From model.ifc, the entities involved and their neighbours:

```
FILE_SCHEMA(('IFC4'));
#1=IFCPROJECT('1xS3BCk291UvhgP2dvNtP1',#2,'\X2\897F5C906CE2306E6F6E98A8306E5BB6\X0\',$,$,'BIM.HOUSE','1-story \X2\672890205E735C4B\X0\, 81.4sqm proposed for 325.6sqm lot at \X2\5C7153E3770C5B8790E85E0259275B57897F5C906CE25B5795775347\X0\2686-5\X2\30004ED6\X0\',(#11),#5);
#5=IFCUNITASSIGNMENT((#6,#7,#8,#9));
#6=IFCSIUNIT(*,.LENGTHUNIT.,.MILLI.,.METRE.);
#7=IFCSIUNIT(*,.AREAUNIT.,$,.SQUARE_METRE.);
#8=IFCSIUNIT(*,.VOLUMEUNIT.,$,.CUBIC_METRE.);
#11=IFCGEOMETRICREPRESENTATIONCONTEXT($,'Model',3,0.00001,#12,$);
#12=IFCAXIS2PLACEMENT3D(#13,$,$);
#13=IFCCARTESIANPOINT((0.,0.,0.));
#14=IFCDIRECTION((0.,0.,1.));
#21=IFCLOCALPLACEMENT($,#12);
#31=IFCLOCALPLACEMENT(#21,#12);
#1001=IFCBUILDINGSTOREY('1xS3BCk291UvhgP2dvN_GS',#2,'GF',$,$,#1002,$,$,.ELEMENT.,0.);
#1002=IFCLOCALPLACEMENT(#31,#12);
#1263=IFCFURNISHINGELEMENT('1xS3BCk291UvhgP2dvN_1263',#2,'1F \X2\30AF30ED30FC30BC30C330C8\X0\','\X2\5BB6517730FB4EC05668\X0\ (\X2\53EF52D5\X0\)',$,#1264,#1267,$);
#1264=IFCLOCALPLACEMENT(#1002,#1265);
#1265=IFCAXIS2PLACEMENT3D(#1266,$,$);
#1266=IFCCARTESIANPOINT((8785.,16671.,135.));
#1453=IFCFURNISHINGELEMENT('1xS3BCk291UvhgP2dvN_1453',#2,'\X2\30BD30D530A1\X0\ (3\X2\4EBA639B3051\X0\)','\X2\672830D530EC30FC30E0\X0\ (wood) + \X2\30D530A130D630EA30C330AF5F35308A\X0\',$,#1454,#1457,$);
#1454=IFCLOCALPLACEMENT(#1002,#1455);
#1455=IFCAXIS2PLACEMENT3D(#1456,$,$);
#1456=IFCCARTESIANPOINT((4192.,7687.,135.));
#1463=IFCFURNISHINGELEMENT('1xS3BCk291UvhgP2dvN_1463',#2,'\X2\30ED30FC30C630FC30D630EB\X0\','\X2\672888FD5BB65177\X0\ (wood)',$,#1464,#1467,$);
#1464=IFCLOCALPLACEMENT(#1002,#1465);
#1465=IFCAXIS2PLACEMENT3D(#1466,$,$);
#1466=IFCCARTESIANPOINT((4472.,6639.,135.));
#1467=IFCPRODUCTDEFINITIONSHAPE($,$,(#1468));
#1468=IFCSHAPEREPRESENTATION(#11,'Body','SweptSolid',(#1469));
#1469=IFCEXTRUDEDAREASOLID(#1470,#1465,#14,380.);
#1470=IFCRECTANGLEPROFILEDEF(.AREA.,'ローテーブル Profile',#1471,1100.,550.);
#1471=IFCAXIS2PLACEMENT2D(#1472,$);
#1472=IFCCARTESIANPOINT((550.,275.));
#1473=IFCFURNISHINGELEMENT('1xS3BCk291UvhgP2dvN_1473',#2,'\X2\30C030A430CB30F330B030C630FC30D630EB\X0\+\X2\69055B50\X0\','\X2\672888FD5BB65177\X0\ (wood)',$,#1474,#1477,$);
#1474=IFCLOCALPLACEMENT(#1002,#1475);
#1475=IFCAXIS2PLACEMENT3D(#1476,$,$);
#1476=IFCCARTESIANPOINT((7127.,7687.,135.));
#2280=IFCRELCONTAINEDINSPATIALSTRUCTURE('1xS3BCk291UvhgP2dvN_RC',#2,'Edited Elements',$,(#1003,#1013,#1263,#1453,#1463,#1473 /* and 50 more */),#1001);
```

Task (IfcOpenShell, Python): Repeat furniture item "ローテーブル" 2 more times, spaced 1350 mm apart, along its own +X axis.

```python
import ifcopenshell
import ifcopenshell.api.geometry
import ifcopenshell.api.root
import ifcopenshell.util.element
import ifcopenshell.util.placement
import ifcopenshell.util.unit

model = ifcopenshell.open("model.ifc")
unit_scale = ifcopenshell.util.unit.calculate_unit_scale(model)


def reuse_history(source, copy):
    """copy_class also copies each property set's owner history, people and application; keep the originals."""
    for rel in copy.IsDefinedBy:
        if rel.is_a("IfcRelDefinesByProperties") and (history := rel.RelatingPropertyDefinition.OwnerHistory):
            rel.RelatingPropertyDefinition.OwnerHistory = source.OwnerHistory
            ifcopenshell.util.element.remove_deep2(model, history)


source = model.by_guid("1xS3BCk291UvhgP2dvN_1463")
base = ifcopenshell.util.placement.get_local_placement(source.ObjectPlacement)
step = base[:3, 0] * 1.35 / unit_scale

for i in range(1, 3):
    copy = ifcopenshell.api.root.copy_class(model, product=source)
    copy.Representation = ifcopenshell.util.element.copy_deep(
        model, source.Representation, exclude=["IfcGeometricRepresentationContext", "IfcRepresentationMap"]
    )
    reuse_history(source, copy)
    matrix = base.copy()
    matrix[:3, 3] += i * step
    print("added at", matrix[:3, 3].round(3) + 0.0)
    ifcopenshell.api.geometry.edit_object_placement(model, product=copy, matrix=matrix, is_si=False)

model.write("model_v2.ifc")
```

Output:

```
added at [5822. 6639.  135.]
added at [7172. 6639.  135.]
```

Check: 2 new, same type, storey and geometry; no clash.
